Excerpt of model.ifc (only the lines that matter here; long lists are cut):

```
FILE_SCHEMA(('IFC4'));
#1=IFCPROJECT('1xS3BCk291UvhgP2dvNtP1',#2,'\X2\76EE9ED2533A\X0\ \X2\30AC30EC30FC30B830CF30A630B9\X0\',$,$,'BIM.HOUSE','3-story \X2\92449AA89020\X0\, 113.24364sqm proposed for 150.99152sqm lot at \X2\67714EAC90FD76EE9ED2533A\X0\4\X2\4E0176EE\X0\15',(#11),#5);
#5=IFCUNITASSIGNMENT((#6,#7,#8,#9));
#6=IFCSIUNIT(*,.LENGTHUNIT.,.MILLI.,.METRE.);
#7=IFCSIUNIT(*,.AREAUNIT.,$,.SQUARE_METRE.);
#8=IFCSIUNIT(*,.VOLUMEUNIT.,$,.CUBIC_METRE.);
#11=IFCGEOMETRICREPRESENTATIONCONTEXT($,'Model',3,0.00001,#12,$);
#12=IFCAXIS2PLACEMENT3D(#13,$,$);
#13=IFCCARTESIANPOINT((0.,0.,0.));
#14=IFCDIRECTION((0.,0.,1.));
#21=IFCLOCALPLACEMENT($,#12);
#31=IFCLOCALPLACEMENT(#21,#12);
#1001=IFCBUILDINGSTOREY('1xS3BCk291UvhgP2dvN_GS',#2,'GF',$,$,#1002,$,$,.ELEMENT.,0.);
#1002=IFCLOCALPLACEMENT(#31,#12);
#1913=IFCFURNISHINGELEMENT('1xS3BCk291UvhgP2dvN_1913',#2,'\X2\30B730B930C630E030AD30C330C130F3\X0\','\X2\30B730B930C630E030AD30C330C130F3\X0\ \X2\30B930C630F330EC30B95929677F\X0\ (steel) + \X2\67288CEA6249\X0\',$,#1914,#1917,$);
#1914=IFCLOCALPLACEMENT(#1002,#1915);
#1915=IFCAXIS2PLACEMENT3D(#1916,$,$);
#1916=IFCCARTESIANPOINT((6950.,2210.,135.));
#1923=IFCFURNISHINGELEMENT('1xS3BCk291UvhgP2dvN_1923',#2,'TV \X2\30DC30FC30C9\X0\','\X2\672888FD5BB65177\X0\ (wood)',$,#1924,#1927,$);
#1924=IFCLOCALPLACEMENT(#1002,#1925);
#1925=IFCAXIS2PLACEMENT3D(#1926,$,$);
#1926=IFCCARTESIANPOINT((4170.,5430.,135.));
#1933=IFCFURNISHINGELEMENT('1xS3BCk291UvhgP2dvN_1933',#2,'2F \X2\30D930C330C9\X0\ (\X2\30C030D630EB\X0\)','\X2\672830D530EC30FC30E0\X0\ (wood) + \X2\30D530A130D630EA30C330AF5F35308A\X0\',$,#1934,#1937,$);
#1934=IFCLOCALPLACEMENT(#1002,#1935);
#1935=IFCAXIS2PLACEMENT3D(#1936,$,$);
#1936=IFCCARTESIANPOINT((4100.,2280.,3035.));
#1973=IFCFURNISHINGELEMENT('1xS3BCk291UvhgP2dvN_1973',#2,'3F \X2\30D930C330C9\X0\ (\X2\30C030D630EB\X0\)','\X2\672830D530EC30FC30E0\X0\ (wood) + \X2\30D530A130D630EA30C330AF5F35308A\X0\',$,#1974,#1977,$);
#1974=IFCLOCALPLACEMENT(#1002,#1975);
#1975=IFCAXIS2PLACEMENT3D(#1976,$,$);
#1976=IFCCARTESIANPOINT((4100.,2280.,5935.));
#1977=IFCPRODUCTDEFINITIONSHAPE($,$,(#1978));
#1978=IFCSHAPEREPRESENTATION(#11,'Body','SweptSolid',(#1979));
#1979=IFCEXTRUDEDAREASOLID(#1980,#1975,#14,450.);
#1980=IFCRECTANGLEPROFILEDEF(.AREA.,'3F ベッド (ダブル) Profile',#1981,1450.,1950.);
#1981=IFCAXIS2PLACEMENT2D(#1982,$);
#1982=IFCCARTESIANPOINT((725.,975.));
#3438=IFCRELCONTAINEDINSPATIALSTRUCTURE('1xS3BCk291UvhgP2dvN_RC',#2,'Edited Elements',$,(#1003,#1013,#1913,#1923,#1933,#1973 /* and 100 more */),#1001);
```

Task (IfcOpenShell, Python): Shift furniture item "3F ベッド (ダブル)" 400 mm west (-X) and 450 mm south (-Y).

```python
import ifcopenshell
import ifcopenshell.api.geometry
import ifcopenshell.util.placement

model = ifcopenshell.open("model.ifc")

item = model.by_guid("1xS3BCk291UvhgP2dvN_1973")
matrix = ifcopenshell.util.placement.get_local_placement(item.ObjectPlacement)
matrix[0, 3] -= 400.0
matrix[1, 3] -= 450.0
ifcopenshell.api.geometry.edit_object_placement(model, product=item, matrix=matrix, is_si=False)

print(ifcopenshell.util.placement.get_local_placement(item.ObjectPlacement).round(3) + 0.0)

model.write("model_edited.ifc")
```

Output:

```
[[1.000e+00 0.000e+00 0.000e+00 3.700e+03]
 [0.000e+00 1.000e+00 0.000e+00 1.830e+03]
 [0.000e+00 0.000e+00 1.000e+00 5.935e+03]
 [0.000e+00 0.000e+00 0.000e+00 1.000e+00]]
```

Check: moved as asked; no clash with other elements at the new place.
